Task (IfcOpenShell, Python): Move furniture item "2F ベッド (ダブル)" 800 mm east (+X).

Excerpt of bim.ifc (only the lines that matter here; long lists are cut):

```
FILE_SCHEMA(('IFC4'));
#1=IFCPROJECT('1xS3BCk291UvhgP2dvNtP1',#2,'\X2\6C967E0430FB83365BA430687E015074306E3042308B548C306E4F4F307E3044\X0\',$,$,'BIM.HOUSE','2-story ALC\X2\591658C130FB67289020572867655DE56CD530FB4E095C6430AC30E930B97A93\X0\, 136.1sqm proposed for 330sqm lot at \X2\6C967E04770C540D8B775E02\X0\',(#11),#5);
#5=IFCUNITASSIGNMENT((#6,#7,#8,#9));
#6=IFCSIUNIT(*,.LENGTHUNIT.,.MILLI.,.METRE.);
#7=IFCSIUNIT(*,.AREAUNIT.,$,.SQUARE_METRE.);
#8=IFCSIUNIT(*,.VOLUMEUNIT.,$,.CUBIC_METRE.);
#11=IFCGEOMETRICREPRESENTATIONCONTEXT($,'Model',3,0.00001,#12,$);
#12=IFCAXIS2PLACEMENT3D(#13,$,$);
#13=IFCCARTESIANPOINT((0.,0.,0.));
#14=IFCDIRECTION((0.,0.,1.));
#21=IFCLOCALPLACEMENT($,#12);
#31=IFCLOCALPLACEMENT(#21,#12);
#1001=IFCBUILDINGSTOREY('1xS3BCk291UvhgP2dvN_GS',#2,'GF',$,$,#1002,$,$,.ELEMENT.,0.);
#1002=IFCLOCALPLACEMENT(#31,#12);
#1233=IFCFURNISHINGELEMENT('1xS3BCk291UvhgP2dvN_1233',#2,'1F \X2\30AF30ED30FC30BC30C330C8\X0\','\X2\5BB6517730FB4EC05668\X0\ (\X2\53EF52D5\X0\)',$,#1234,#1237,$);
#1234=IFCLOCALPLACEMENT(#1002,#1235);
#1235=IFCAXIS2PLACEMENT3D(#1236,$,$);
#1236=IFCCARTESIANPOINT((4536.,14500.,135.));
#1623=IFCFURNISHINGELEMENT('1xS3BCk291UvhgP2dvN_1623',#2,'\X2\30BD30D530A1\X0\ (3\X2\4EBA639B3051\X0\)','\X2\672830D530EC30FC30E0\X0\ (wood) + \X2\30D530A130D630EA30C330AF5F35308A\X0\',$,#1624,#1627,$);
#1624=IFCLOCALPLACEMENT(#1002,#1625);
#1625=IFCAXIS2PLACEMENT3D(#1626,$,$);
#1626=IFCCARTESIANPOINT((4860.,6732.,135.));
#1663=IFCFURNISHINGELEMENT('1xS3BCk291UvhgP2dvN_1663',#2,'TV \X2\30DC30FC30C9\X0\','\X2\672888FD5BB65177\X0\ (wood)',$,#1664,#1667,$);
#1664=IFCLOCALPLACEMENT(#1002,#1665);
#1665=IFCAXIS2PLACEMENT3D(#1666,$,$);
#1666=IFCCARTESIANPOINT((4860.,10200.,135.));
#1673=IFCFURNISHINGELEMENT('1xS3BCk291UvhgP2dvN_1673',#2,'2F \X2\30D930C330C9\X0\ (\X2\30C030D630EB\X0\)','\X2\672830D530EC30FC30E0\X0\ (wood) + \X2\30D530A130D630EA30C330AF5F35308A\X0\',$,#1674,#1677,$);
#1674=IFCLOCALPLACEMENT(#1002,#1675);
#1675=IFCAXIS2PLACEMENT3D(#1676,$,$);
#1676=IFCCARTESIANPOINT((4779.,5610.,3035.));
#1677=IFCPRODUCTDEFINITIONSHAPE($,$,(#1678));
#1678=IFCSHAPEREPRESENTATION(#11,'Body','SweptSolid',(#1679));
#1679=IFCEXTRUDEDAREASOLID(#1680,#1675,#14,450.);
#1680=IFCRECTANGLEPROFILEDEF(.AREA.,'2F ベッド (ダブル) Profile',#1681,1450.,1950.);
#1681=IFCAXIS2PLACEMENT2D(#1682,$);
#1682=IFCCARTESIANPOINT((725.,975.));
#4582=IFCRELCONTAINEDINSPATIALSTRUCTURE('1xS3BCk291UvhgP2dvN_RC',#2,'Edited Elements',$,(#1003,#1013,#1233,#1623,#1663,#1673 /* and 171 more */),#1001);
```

```python
import ifcopenshell
import ifcopenshell.api.geometry
import ifcopenshell.util.placement

model = ifcopenshell.open("bim.ifc")

item = model.by_id(1673)
matrix = ifcopenshell.util.placement.get_local_placement(item.ObjectPlacement)
matrix[0, 3] += 800.0
ifcopenshell.api.geometry.edit_object_placement(model, product=item, matrix=matrix, is_si=False)

print(ifcopenshell.util.placement.get_local_placement(item.ObjectPlacement).round(3) + 0.0)

model.write("bim-out.ifc")
```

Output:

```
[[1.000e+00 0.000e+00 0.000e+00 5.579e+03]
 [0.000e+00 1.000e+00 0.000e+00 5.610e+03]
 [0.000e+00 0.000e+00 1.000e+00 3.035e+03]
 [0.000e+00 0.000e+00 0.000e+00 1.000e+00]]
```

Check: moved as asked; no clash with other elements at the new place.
